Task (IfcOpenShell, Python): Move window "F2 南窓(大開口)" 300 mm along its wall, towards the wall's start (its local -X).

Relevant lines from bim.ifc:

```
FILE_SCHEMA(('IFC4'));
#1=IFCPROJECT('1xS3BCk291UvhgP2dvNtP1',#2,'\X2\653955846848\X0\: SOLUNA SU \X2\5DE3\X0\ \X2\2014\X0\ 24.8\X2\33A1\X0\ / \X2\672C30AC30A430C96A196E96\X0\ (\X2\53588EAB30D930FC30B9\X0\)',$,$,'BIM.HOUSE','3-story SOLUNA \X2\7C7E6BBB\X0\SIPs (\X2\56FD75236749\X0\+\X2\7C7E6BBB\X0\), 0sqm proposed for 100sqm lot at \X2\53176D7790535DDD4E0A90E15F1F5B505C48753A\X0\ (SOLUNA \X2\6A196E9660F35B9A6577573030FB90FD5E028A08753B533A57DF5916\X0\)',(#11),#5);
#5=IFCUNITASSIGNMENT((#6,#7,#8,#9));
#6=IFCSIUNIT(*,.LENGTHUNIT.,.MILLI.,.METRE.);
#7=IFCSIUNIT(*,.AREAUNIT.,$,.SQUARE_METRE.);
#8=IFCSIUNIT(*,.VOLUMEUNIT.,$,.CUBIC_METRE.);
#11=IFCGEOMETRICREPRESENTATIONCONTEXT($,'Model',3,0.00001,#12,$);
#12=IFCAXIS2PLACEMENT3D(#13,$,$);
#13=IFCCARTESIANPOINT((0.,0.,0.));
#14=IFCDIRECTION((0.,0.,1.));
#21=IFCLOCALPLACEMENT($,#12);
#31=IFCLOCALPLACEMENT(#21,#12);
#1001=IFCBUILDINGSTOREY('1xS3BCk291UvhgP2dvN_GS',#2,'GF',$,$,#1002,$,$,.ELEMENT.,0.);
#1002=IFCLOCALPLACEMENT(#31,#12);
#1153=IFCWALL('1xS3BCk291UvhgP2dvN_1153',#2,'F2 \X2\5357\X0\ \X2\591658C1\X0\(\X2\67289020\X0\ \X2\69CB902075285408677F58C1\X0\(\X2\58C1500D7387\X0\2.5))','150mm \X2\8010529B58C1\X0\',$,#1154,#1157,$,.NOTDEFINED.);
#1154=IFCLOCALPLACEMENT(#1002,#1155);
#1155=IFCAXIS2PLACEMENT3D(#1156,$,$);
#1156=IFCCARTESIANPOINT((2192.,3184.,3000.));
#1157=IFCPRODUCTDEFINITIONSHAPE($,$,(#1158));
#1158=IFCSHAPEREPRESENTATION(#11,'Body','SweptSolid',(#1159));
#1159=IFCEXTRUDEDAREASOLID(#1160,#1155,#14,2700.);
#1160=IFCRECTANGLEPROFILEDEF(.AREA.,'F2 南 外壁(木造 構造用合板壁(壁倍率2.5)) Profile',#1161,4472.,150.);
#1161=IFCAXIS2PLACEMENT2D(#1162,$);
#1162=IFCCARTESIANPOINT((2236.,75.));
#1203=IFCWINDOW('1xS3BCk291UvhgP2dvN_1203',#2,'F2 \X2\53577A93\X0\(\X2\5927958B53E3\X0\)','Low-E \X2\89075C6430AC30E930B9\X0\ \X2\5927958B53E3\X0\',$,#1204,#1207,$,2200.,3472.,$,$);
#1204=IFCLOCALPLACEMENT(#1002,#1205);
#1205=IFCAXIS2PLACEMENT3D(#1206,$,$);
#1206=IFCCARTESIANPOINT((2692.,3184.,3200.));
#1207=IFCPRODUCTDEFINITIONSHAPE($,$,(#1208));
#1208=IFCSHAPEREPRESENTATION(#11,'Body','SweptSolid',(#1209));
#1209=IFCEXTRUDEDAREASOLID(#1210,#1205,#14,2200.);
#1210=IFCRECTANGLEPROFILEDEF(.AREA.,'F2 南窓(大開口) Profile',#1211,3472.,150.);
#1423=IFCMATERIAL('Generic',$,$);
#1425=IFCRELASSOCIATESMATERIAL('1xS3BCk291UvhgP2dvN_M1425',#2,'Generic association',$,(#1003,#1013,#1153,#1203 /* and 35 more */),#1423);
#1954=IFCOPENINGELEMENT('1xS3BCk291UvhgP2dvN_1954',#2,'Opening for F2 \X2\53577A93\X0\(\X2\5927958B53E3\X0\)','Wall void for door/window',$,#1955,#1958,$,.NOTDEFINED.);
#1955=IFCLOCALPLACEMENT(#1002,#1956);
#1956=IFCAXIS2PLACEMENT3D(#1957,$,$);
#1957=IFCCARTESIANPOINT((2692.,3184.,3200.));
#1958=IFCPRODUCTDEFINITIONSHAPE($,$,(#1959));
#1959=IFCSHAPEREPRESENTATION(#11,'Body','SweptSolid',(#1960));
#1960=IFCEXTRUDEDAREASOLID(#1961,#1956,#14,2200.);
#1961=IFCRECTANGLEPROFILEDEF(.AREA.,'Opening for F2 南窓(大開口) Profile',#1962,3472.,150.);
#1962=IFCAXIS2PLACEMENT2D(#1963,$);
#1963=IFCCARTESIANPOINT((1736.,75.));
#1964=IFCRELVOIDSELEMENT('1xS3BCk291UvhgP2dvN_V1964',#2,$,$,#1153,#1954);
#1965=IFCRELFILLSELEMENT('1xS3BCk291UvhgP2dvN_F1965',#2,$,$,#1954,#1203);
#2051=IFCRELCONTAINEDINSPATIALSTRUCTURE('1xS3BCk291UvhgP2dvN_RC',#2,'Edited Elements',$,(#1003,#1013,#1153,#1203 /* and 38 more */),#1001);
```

```python
import ifcopenshell
import ifcopenshell.api.geometry
import ifcopenshell.util.placement
import ifcopenshell.util.unit

model = ifcopenshell.open("bim.ifc")
unit_scale = ifcopenshell.util.unit.calculate_unit_scale(model)

window = model.by_guid("1xS3BCk291UvhgP2dvN_1203")
opening = window.FillsVoids[0].RelatingOpeningElement
wall = opening.VoidsElements[0].RelatingBuildingElement

wall_matrix = ifcopenshell.util.placement.get_local_placement(wall.ObjectPlacement)
shift = wall_matrix[:3, 0] * -0.3 / unit_scale
before = ifcopenshell.util.placement.get_local_placement(window.ObjectPlacement)[:3, 3].copy()

# The window is not placed relative to its opening, so move both.
for product in (opening, window):
    matrix = ifcopenshell.util.placement.get_local_placement(product.ObjectPlacement)
    matrix[:3, 3] += shift
    ifcopenshell.api.geometry.edit_object_placement(model, product=product, matrix=matrix, is_si=False)

after = ifcopenshell.util.placement.get_local_placement(window.ObjectPlacement)[:3, 3]
print("window moved by", (after - before).round(3) + 0.0)

model.write("bim_rev.ifc")
```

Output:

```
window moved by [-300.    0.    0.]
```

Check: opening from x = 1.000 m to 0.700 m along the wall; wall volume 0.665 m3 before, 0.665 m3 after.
